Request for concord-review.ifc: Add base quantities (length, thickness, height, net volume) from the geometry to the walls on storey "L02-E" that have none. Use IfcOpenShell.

First a look at what the model holds.

```python
import ifcopenshell
import ifcopenshell.util.element
import ifcopenshell.util.unit

model = ifcopenshell.open("concord-review.ifc")
print(model.schema)
for unit_type in ("LENGTHUNIT", "AREAUNIT", "VOLUMEUNIT"):
    print(unit_type, ifcopenshell.util.unit.calculate_unit_scale(model, unit_type))
storey = next(s for s in model.by_type("IfcBuildingStorey") if s.Name == "L02-E")
walls = [e for e in ifcopenshell.util.element.get_decomposition(storey) if e.is_a("IfcWall")]
for e in sorted(walls, key=lambda e: e.id()):
    print(e.id(), e.is_a(), e.Name, list(ifcopenshell.util.element.get_psets(e, qtos_only=True)), sep=" | ")
```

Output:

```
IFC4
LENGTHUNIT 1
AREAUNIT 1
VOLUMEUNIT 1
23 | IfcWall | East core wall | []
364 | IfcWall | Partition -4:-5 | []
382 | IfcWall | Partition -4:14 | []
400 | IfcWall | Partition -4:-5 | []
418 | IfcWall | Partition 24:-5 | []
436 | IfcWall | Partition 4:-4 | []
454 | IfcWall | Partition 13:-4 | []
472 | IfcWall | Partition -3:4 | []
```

```python
import ifcopenshell
import ifcopenshell.api.pset
import ifcopenshell.geom
import ifcopenshell.util.element
import ifcopenshell.util.shape
import ifcopenshell.util.unit

model = ifcopenshell.open("concord-review.ifc")
unit_scale = ifcopenshell.util.unit.calculate_unit_scale(model)
volume_scale = ifcopenshell.util.unit.calculate_unit_scale(model, "VOLUMEUNIT")
settings = ifcopenshell.geom.settings()

storey = next(s for s in model.by_type("IfcBuildingStorey") if s.Name == "L02-E")
walls = [e for e in ifcopenshell.util.element.get_decomposition(storey) if e.is_a("IfcWall")]

for e in sorted(walls, key=lambda e: e.id()):
    if ifcopenshell.util.element.get_psets(e, qtos_only=True, should_inherit=False):
        continue
    # Geometry comes back in metres, in the element's own axes.
    shape = ifcopenshell.geom.create_shape(settings, e)
    values = {
        "Length": ifcopenshell.util.shape.get_x(shape.geometry) / unit_scale,
        "Width": ifcopenshell.util.shape.get_y(shape.geometry) / unit_scale,
        "Height": ifcopenshell.util.shape.get_z(shape.geometry) / unit_scale,
        "NetVolume": ifcopenshell.util.shape.get_volume(shape.geometry) / volume_scale,
    }
    qto = ifcopenshell.api.pset.add_qto(model, product=e, name="Qto_WallBaseQuantities")
    ifcopenshell.api.pset.edit_qto(model, qto=qto, properties=values)
    print(e.id(), {k: round(v, 3) for k, v in values.items()})

model.write("concord-review_v2.ifc")
```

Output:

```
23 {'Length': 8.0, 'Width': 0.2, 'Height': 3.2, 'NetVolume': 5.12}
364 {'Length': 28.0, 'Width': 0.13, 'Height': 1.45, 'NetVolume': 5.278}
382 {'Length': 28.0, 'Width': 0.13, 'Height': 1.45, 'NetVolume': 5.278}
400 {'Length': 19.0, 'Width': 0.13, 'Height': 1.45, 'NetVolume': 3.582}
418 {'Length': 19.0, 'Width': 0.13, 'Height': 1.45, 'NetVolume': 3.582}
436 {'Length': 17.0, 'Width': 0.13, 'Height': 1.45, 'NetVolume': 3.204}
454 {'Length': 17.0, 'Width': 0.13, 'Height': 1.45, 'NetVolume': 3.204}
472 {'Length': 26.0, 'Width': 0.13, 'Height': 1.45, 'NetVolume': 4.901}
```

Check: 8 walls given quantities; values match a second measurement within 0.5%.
